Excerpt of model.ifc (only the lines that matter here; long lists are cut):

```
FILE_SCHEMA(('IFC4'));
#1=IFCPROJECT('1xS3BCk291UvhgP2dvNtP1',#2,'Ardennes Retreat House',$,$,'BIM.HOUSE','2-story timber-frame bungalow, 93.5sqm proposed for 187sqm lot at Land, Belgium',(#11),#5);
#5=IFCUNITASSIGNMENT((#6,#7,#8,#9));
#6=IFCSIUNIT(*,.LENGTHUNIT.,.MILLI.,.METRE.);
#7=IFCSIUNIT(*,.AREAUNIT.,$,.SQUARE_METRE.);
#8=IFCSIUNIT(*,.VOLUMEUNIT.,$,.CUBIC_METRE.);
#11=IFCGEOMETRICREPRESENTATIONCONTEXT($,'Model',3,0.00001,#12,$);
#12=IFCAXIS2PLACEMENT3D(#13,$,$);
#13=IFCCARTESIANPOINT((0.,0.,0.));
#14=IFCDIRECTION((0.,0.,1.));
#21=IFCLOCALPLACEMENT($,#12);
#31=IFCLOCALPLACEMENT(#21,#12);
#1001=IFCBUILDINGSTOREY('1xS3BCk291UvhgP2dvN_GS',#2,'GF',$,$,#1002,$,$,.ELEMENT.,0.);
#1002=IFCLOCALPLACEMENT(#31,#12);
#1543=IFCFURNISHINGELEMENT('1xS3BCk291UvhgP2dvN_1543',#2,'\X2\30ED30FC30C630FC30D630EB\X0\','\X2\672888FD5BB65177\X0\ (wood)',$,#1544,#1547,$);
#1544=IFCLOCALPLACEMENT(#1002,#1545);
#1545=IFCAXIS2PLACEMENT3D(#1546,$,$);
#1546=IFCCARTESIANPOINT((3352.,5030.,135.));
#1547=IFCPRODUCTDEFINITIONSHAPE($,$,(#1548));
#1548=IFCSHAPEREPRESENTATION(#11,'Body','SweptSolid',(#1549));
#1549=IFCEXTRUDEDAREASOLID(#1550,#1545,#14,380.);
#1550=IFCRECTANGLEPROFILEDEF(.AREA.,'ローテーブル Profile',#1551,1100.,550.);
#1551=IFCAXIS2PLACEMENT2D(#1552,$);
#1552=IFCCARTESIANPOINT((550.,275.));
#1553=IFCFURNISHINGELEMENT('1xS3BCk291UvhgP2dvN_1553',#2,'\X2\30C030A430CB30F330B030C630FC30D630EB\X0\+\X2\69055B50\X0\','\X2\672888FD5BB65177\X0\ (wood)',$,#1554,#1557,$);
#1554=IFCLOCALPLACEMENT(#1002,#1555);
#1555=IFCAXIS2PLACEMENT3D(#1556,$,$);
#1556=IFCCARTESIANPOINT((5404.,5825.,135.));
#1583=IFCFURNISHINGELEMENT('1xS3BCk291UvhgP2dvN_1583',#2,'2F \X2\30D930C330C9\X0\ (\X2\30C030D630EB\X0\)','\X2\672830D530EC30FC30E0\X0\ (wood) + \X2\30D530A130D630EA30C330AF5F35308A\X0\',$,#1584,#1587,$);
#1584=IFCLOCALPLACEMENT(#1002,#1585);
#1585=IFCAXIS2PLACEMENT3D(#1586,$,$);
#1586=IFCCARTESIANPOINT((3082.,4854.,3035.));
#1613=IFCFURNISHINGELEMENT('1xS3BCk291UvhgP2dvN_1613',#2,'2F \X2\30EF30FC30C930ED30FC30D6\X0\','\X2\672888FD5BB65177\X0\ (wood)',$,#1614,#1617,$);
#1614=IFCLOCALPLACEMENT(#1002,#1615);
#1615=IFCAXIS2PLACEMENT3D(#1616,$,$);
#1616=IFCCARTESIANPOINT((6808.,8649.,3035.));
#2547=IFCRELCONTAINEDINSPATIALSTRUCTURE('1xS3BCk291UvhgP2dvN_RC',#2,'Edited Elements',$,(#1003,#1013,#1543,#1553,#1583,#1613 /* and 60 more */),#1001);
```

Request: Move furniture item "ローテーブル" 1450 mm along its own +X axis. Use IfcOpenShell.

```python
import ifcopenshell
import ifcopenshell.api.geometry
import ifcopenshell.util.placement

model = ifcopenshell.open("model.ifc")

item = model.by_id(1543)
matrix = ifcopenshell.util.placement.get_local_placement(item.ObjectPlacement)
matrix[:3, 3] += matrix[:3, 0] * 1450.0
ifcopenshell.api.geometry.edit_object_placement(model, product=item, matrix=matrix, is_si=False)

print(ifcopenshell.util.placement.get_local_placement(item.ObjectPlacement).round(3) + 0.0)

model.write("model_rev.ifc")
```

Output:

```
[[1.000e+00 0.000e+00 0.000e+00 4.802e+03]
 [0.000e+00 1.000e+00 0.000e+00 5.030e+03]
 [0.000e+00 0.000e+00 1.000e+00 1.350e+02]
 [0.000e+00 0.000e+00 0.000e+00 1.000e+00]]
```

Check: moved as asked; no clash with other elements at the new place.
